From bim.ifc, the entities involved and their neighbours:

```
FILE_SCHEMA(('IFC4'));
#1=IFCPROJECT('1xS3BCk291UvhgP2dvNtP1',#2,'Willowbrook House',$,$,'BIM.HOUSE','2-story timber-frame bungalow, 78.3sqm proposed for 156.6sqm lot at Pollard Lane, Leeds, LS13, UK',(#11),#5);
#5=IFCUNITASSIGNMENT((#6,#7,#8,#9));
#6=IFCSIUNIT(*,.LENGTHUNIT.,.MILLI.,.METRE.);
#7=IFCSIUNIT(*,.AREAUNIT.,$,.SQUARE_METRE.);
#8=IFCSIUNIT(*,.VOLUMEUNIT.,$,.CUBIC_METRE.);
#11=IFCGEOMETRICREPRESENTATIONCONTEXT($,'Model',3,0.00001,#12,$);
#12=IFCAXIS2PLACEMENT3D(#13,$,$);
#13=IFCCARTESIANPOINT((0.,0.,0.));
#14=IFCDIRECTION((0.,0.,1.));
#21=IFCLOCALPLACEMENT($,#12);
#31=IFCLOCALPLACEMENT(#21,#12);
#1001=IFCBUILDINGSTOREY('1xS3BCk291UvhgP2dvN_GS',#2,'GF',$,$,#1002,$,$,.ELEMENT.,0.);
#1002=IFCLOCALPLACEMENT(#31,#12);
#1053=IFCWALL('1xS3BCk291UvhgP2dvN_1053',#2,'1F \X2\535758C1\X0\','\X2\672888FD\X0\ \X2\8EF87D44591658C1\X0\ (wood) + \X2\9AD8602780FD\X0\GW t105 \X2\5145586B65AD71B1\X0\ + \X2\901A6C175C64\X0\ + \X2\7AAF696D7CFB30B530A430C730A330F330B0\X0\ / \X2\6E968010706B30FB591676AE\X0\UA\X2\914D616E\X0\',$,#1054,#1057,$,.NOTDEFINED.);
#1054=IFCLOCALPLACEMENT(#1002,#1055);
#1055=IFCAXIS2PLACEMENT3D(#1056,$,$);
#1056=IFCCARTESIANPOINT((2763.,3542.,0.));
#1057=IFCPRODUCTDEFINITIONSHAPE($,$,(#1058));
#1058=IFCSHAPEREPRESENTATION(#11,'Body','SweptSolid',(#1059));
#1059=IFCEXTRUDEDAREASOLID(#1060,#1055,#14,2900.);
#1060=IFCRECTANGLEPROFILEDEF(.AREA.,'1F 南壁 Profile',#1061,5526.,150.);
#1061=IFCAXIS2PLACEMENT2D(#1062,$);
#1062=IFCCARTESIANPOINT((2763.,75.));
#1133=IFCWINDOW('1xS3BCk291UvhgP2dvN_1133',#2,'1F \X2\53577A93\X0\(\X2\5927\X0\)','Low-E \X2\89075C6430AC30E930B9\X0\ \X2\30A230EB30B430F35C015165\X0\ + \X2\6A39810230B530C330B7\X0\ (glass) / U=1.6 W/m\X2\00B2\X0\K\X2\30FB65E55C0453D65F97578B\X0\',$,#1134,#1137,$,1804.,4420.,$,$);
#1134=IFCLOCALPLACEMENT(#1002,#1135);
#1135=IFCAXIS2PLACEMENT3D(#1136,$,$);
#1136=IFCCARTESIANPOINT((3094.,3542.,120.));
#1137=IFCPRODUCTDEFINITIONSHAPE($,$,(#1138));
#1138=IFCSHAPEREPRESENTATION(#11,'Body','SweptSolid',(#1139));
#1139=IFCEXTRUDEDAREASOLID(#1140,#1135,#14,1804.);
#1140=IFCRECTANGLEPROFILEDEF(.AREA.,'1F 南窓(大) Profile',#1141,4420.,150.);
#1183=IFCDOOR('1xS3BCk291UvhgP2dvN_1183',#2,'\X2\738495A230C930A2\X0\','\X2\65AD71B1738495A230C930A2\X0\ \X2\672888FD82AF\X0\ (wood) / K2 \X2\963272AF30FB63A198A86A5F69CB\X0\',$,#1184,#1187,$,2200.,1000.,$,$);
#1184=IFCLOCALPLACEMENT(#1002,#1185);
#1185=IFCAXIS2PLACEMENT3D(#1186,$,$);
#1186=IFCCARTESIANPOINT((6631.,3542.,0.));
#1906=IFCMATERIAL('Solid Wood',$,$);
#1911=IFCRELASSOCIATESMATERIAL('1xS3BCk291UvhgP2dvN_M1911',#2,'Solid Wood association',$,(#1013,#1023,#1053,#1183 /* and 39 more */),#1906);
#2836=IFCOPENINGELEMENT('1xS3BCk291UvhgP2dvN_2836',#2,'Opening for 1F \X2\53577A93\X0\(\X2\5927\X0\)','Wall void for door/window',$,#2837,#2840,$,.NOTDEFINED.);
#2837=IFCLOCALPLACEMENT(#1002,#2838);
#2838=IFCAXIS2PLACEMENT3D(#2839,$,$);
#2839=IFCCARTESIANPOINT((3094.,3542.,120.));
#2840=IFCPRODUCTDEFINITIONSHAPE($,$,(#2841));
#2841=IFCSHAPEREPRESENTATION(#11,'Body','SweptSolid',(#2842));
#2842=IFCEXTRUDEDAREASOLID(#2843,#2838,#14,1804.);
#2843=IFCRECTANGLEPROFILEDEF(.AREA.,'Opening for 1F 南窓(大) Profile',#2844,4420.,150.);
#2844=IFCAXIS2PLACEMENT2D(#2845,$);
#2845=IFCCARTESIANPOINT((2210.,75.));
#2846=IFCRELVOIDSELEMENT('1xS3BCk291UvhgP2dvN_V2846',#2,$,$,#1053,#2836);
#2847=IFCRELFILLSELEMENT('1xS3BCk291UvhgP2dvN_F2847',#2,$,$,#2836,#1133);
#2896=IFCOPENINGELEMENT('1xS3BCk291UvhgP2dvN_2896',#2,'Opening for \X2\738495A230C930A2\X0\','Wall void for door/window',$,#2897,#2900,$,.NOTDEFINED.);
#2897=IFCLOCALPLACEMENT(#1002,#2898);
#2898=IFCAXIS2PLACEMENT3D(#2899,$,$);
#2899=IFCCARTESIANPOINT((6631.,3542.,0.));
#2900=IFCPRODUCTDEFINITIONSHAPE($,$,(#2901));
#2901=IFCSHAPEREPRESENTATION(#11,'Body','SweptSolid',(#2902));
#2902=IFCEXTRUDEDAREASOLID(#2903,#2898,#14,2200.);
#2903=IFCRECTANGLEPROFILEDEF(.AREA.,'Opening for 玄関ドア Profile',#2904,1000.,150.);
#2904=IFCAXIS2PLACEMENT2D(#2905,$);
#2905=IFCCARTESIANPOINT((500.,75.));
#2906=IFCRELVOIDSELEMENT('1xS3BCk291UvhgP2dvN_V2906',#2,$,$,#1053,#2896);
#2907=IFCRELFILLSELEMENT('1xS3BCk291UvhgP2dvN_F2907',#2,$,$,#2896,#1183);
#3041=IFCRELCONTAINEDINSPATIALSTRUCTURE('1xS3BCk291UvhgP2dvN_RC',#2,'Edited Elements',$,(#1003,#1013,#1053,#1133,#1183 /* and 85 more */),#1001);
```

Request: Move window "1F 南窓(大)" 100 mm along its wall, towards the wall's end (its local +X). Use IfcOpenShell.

```python
import ifcopenshell
import ifcopenshell.api.geometry
import ifcopenshell.util.placement
import ifcopenshell.util.unit

model = ifcopenshell.open("bim.ifc")
unit_scale = ifcopenshell.util.unit.calculate_unit_scale(model)

window = model.by_guid("1xS3BCk291UvhgP2dvN_1133")
opening = window.FillsVoids[0].RelatingOpeningElement
wall = opening.VoidsElements[0].RelatingBuildingElement

wall_matrix = ifcopenshell.util.placement.get_local_placement(wall.ObjectPlacement)
shift = wall_matrix[:3, 0] * 0.1 / unit_scale
before = ifcopenshell.util.placement.get_local_placement(window.ObjectPlacement)[:3, 3].copy()

# The window is not placed relative to its opening, so move both.
for product in (opening, window):
    matrix = ifcopenshell.util.placement.get_local_placement(product.ObjectPlacement)
    matrix[:3, 3] += shift
    ifcopenshell.api.geometry.edit_object_placement(model, product=product, matrix=matrix, is_si=False)

after = ifcopenshell.util.placement.get_local_placement(window.ObjectPlacement)[:3, 3]
print("window moved by", (after - before).round(3) + 0.0)

model.write("bim_updated.ifc")
```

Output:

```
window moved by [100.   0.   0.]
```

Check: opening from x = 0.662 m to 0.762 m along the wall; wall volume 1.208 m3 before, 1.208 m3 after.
